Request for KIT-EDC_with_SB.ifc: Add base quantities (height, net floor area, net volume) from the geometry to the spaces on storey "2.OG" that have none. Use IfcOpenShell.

First a look at what the model holds.

```python
import ifcopenshell
import ifcopenshell.util.element
import ifcopenshell.util.unit

model = ifcopenshell.open("KIT-EDC_with_SB.ifc")
print(model.schema)
for unit_type in ("LENGTHUNIT", "AREAUNIT", "VOLUMEUNIT"):
    print(unit_type, ifcopenshell.util.unit.calculate_unit_scale(model, unit_type))
storey = next(s for s in model.by_type("IfcBuildingStorey") if s.Name == "2.OG")
spaces = [e for e in ifcopenshell.util.element.get_decomposition(storey) if e.is_a("IfcSpace")]
for e in sorted(spaces, key=lambda e: e.id()):
    print(e.id(), e.is_a(), e.Name, list(ifcopenshell.util.element.get_psets(e, qtos_only=True)), sep=" | ")
```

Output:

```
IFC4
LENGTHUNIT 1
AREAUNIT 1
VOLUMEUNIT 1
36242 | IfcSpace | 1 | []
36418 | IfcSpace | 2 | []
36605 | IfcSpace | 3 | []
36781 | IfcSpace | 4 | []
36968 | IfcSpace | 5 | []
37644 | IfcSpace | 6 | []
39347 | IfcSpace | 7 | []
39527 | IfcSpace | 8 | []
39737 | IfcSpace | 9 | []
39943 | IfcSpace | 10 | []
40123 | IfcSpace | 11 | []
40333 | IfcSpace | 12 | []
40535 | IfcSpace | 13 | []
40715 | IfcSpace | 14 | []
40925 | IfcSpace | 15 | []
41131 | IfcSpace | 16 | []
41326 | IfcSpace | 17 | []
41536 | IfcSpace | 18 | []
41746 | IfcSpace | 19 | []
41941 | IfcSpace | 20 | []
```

```python
import ifcopenshell
import ifcopenshell.api.pset
import ifcopenshell.geom
import ifcopenshell.util.element
import ifcopenshell.util.shape
import ifcopenshell.util.unit

model = ifcopenshell.open("KIT-EDC_with_SB.ifc")
unit_scale = ifcopenshell.util.unit.calculate_unit_scale(model)
area_scale = ifcopenshell.util.unit.calculate_unit_scale(model, "AREAUNIT")
volume_scale = ifcopenshell.util.unit.calculate_unit_scale(model, "VOLUMEUNIT")
settings = ifcopenshell.geom.settings()

storey = next(s for s in model.by_type("IfcBuildingStorey") if s.Name == "2.OG")
spaces = [e for e in ifcopenshell.util.element.get_decomposition(storey) if e.is_a("IfcSpace")]

for e in sorted(spaces, key=lambda e: e.id()):
    if ifcopenshell.util.element.get_psets(e, qtos_only=True, should_inherit=False):
        continue
    # Geometry comes back in metres, in the element's own axes.
    shape = ifcopenshell.geom.create_shape(settings, e)
    values = {
        "Height": ifcopenshell.util.shape.get_z(shape.geometry) / unit_scale,
        "NetFloorArea": ifcopenshell.util.shape.get_footprint_area(shape.geometry) / area_scale,
        "NetVolume": ifcopenshell.util.shape.get_volume(shape.geometry) / volume_scale,
    }
    qto = ifcopenshell.api.pset.add_qto(model, product=e, name="Qto_SpaceBaseQuantities")
    ifcopenshell.api.pset.edit_qto(model, qto=qto, properties=values)
    print(e.id(), {k: round(v, 3) for k, v in values.items()})

model.write("KIT-EDC_with_SB_v2.ifc")
```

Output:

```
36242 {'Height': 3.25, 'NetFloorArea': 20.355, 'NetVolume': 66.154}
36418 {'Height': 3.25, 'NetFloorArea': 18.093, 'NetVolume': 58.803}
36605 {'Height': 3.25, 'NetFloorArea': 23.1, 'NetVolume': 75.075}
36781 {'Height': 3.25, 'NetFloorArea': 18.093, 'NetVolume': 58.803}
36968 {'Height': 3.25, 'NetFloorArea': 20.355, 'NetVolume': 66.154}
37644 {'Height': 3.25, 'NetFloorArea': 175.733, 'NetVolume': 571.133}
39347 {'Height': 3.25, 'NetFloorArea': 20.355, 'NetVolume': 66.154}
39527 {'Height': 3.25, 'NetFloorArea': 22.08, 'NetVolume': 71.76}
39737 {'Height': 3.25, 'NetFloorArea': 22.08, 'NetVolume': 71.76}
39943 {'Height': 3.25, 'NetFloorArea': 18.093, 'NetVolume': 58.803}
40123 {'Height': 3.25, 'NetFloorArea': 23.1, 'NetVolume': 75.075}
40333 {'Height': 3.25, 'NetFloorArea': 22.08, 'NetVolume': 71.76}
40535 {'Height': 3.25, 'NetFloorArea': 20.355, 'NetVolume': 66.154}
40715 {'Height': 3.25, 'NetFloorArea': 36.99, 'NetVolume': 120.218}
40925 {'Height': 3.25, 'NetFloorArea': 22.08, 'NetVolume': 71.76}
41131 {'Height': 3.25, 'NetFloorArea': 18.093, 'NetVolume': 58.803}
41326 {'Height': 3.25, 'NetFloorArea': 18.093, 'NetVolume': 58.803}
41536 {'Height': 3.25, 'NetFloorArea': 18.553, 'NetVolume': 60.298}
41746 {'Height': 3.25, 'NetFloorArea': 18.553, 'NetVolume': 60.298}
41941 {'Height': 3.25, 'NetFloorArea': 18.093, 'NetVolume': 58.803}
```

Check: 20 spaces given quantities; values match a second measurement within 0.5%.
